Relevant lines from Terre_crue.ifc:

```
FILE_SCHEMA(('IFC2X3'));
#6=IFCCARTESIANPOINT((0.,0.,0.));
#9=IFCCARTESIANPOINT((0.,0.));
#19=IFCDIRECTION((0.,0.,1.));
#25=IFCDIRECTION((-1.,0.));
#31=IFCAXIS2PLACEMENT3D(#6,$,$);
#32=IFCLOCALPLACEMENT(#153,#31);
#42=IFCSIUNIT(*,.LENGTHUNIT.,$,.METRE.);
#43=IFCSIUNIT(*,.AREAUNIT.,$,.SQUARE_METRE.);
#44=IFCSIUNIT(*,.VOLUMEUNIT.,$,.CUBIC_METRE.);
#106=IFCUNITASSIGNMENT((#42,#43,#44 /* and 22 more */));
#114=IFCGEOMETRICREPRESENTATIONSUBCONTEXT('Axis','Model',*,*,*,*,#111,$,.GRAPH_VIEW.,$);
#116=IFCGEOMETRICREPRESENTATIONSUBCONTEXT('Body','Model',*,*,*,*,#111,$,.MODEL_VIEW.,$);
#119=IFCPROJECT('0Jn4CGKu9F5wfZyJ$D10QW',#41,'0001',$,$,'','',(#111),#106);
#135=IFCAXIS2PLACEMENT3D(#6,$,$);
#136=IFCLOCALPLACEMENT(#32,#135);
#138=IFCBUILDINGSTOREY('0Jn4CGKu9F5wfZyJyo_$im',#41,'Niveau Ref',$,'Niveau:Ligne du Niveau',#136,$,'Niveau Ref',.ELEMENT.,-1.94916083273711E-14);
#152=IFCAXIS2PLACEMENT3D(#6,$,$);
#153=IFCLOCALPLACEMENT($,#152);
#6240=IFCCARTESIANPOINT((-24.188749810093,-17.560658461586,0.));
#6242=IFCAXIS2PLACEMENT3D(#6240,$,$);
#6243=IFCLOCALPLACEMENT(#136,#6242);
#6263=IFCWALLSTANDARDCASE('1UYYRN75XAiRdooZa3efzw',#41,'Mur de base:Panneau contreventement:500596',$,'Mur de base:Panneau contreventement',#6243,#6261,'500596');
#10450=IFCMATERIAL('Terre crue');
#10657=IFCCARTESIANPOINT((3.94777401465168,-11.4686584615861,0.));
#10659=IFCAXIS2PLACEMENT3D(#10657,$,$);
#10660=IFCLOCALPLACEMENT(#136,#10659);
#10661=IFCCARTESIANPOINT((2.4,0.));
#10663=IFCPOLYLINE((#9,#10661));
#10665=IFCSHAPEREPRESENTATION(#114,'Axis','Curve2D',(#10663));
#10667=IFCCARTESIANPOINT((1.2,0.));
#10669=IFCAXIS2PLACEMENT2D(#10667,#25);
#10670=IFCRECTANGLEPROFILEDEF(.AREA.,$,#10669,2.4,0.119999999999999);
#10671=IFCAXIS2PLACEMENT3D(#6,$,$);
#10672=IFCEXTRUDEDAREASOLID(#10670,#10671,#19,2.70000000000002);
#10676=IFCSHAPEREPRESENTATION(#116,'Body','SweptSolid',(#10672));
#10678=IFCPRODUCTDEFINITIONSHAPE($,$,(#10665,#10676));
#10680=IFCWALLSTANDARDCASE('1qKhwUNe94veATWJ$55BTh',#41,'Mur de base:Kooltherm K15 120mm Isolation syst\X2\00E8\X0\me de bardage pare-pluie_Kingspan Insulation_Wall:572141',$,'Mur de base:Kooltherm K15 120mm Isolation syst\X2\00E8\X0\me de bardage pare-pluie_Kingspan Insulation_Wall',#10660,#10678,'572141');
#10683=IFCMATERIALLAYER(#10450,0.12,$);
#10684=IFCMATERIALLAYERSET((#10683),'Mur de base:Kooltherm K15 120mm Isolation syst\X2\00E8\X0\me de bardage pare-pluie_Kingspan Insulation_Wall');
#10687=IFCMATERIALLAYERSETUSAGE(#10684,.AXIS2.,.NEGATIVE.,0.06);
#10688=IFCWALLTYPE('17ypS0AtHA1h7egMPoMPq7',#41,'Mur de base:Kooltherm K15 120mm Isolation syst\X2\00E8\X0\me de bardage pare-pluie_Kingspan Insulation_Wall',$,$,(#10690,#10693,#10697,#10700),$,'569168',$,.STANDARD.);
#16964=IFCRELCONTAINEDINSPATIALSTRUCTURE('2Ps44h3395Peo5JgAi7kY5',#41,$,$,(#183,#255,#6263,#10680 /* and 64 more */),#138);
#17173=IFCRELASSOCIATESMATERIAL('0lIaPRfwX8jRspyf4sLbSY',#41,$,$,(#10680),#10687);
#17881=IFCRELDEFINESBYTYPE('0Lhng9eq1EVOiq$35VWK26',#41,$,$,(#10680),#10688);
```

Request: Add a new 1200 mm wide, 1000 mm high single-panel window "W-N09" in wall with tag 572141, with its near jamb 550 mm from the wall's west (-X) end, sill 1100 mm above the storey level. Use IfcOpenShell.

```python
import numpy as np
import ifcopenshell
import ifcopenshell.api.feature
import ifcopenshell.api.geometry
import ifcopenshell.api.root
import ifcopenshell.api.spatial
import ifcopenshell.api.type
import ifcopenshell.geom
import ifcopenshell.util.element
import ifcopenshell.util.placement
import ifcopenshell.util.representation
import ifcopenshell.util.shape
import ifcopenshell.util.unit

model = ifcopenshell.open("Terre_crue.ifc")
unit_scale = ifcopenshell.util.unit.calculate_unit_scale(model)
settings = ifcopenshell.geom.settings()


def volume(element):
    """Net volume in cubic metres, openings subtracted."""
    shape = ifcopenshell.geom.create_shape(settings, element)
    return ifcopenshell.util.shape.get_volume(shape.geometry)


wall = model.by_id(10680)
storey = ifcopenshell.util.element.get_container(wall, ifc_class="IfcBuildingStorey")
context = ifcopenshell.util.representation.get_context(model, "Model", "Body", "MODEL_VIEW")
before = volume(wall)

width, height, from_end, sill = 1.2, 1, 0.55, 1.1  # metres

# The wall runs along its own X axis, and the end named is its -X end.
wall_shape = ifcopenshell.geom.create_shape(settings, wall)
x, y, z = ifcopenshell.util.shape.get_vertices(wall_shape.geometry).T
start = x.min() + from_end
face, thickness = float(y.min()), float(y.max() - y.min())
wall_matrix = ifcopenshell.util.placement.get_local_placement(wall.ObjectPlacement)
level = ifcopenshell.util.placement.get_local_placement(storey.ObjectPlacement)[2, 3]


def in_wall(x, y):
    """Placement at x, y metres in the wall's axes, at sill height."""
    matrix = wall_matrix.copy()
    matrix[:, 3] = wall_matrix @ np.array([x / unit_scale, y / unit_scale, 0.0, 1.0])
    matrix[2, 3] = level + sill / unit_scale
    return matrix


# Opening: a box that overshoots both wall faces by 50 mm.
opening = ifcopenshell.api.root.create_entity(model, ifc_class="IfcOpeningElement")
box = ifcopenshell.api.geometry.add_wall_representation(
    model, context=context, length=width, height=height, thickness=thickness + 0.1
)
ifcopenshell.api.geometry.assign_representation(model, product=opening, representation=box)
ifcopenshell.api.geometry.edit_object_placement(model, product=opening, matrix=in_wall(start, face - 0.05), is_si=False)
ifcopenshell.api.feature.add_feature(model, feature=opening, element=wall)

window = ifcopenshell.api.root.create_entity(model, ifc_class="IfcWindow", name="W-N09")
window.OverallWidth, window.OverallHeight = width / unit_scale, height / unit_scale
body = ifcopenshell.api.geometry.add_window_representation(
    model,
    context=context,
    overall_width=window.OverallWidth,
    overall_height=window.OverallHeight,
    partition_type="SINGLE_PANEL",
)
ifcopenshell.api.geometry.assign_representation(model, product=window, representation=body)
ifcopenshell.api.spatial.assign_container(model, products=[window], relating_structure=storey)
fills = ifcopenshell.api.feature.add_filling(model, opening=opening, element=window)
fills.OwnerHistory = window.OwnerHistory  # required in IFC2X3

# IFC2X3 keeps the operation on the window style.
style = ifcopenshell.api.root.create_entity(model, ifc_class="IfcWindowStyle", name="W-N09")
style.OperationType, style.ConstructionType = "SINGLE_PANEL", "NOTDEFINED"
style.ParameterTakesPrecedence = style.Sizeable = False
ifcopenshell.api.type.assign_type(model, related_objects=[window], relating_type=style)

# Centre the window in the wall's thickness.
ifcopenshell.api.geometry.edit_object_placement(model, product=window, matrix=in_wall(start, face), is_si=False)
window_shape = ifcopenshell.geom.create_shape(settings, window)
depth = ifcopenshell.util.shape.get_vertices(window_shape.geometry)[:, 1]
offset = face + thickness / 2 - (depth.min() + depth.max()) / 2
ifcopenshell.api.geometry.edit_object_placement(model, product=window, matrix=in_wall(start, offset), is_si=False)

after = volume(wall)

print(f"wall volume {before:.3f} -> {after:.3f} m3")

model.write("Terre_crue_edited.ifc")
```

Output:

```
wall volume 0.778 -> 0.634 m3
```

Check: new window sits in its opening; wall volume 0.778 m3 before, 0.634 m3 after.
